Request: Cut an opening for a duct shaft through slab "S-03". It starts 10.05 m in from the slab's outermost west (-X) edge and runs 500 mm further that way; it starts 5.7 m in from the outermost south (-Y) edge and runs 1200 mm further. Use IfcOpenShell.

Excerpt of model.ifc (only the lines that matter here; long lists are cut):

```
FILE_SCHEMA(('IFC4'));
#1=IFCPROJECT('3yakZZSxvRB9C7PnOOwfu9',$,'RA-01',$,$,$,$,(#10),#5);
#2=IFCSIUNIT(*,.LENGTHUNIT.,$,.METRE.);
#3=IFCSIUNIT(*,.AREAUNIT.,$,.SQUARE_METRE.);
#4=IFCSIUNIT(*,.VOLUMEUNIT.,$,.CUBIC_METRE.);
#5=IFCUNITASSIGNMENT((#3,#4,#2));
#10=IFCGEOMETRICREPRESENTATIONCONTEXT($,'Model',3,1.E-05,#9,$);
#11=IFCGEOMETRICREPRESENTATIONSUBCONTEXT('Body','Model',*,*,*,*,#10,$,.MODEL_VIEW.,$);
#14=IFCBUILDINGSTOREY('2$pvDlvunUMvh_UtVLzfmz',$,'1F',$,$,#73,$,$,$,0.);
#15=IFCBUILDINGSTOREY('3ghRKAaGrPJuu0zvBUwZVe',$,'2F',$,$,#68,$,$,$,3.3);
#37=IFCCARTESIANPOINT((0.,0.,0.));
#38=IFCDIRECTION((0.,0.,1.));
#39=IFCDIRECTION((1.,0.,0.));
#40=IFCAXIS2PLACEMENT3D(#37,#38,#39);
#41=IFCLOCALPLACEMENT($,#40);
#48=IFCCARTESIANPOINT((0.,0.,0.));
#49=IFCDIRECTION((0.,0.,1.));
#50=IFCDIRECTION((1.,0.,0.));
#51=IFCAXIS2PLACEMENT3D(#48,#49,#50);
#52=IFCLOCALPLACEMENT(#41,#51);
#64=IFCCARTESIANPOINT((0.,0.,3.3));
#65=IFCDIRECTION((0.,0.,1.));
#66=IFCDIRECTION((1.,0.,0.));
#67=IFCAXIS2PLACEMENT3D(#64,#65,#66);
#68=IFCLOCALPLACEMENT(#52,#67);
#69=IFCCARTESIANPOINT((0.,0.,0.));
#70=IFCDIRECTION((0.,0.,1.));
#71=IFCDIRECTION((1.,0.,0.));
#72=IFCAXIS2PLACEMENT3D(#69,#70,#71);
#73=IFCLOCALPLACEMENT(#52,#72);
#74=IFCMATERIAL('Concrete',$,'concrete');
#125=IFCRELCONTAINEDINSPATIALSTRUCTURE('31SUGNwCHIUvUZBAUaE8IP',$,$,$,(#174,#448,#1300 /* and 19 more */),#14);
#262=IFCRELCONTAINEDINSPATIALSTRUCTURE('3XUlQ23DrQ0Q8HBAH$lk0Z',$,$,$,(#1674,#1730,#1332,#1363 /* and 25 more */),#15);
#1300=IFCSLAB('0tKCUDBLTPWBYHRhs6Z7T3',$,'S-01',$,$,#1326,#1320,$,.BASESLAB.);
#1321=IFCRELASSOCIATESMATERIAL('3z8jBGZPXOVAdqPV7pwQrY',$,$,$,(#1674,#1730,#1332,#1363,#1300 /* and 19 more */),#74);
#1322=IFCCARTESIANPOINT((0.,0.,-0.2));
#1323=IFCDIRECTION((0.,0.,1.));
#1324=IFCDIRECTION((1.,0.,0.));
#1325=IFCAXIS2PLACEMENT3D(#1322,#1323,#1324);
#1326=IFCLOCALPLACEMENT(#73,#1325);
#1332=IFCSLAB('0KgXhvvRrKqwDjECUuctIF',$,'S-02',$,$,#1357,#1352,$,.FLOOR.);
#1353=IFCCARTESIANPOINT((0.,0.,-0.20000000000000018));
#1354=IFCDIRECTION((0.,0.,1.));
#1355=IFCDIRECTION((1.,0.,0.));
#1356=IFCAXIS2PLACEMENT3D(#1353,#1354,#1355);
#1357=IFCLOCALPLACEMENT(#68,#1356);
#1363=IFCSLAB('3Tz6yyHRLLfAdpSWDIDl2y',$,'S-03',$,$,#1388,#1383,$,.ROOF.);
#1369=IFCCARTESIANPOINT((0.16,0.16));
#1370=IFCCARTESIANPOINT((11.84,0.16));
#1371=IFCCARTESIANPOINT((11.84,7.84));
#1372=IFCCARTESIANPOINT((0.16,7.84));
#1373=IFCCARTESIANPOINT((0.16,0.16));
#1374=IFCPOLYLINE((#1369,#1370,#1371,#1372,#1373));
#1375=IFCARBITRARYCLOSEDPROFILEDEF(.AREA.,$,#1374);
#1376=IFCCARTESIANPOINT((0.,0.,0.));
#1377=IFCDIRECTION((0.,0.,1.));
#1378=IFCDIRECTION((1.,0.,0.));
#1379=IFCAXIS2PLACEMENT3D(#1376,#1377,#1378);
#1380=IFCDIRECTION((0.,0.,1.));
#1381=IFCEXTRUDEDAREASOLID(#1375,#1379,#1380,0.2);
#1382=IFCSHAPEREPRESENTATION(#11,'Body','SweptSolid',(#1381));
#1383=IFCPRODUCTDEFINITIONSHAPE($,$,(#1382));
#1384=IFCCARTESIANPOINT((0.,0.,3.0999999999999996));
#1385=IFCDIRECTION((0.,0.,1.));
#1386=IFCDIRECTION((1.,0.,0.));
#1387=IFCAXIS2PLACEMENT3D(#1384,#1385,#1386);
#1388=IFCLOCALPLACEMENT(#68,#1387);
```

```python
import numpy as np
import ifcopenshell
import ifcopenshell.api.feature
import ifcopenshell.api.geometry
import ifcopenshell.api.root
import ifcopenshell.geom
import ifcopenshell.util.placement
import ifcopenshell.util.representation
import ifcopenshell.util.shape
import ifcopenshell.util.unit

model = ifcopenshell.open("model.ifc")
unit_scale = ifcopenshell.util.unit.calculate_unit_scale(model)
settings = ifcopenshell.geom.settings()


def volume(element):
    """Net volume in cubic metres, openings subtracted."""
    shape = ifcopenshell.geom.create_shape(settings, element)
    return ifcopenshell.util.shape.get_volume(shape.geometry)


slab = model.by_guid("3Tz6yyHRLLfAdpSWDIDl2y")
before = volume(slab)

# Extent in the slab's own axes, in metres. The edges named are its -X and -Y sides.
slab_shape = ifcopenshell.geom.create_shape(settings, slab)
vertices = ifcopenshell.util.shape.get_vertices(slab_shape.geometry)
x_min, y_min, bottom = vertices.min(axis=0)
top = vertices[:, 2].max()

opening = ifcopenshell.api.root.create_entity(model, ifc_class="IfcOpeningElement", name="Duct shaft opening", predefined_type="OPENING")
context = ifcopenshell.util.representation.get_context(model, "Model", "Body", "MODEL_VIEW")
width, depth = 0.5, 1.2
outline = [(0.0, 0.0), (width, 0.0), (width, depth), (0.0, depth), (0.0, 0.0)]
# Overshoot both faces by 50 mm so the cut is clean.
shape = ifcopenshell.api.geometry.add_slab_representation(
    model, context=context, depth=top - bottom + 0.1, polyline=outline
)
ifcopenshell.api.geometry.assign_representation(model, product=opening, representation=shape)

matrix = ifcopenshell.util.placement.get_local_placement(slab.ObjectPlacement)
matrix[:, 3] = matrix @ np.append(np.array([x_min + 10.05, y_min + 5.7, bottom - 0.05]) / unit_scale, 1.0)
ifcopenshell.api.geometry.edit_object_placement(model, product=opening, matrix=matrix, is_si=False)
ifcopenshell.api.feature.add_feature(model, feature=opening, element=slab)

after = volume(slab)

print(f"slab volume {before:.3f} -> {after:.3f} m3")

model.write("model_updated.ifc")
```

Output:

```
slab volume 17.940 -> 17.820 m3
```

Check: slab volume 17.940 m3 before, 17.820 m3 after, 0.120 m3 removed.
